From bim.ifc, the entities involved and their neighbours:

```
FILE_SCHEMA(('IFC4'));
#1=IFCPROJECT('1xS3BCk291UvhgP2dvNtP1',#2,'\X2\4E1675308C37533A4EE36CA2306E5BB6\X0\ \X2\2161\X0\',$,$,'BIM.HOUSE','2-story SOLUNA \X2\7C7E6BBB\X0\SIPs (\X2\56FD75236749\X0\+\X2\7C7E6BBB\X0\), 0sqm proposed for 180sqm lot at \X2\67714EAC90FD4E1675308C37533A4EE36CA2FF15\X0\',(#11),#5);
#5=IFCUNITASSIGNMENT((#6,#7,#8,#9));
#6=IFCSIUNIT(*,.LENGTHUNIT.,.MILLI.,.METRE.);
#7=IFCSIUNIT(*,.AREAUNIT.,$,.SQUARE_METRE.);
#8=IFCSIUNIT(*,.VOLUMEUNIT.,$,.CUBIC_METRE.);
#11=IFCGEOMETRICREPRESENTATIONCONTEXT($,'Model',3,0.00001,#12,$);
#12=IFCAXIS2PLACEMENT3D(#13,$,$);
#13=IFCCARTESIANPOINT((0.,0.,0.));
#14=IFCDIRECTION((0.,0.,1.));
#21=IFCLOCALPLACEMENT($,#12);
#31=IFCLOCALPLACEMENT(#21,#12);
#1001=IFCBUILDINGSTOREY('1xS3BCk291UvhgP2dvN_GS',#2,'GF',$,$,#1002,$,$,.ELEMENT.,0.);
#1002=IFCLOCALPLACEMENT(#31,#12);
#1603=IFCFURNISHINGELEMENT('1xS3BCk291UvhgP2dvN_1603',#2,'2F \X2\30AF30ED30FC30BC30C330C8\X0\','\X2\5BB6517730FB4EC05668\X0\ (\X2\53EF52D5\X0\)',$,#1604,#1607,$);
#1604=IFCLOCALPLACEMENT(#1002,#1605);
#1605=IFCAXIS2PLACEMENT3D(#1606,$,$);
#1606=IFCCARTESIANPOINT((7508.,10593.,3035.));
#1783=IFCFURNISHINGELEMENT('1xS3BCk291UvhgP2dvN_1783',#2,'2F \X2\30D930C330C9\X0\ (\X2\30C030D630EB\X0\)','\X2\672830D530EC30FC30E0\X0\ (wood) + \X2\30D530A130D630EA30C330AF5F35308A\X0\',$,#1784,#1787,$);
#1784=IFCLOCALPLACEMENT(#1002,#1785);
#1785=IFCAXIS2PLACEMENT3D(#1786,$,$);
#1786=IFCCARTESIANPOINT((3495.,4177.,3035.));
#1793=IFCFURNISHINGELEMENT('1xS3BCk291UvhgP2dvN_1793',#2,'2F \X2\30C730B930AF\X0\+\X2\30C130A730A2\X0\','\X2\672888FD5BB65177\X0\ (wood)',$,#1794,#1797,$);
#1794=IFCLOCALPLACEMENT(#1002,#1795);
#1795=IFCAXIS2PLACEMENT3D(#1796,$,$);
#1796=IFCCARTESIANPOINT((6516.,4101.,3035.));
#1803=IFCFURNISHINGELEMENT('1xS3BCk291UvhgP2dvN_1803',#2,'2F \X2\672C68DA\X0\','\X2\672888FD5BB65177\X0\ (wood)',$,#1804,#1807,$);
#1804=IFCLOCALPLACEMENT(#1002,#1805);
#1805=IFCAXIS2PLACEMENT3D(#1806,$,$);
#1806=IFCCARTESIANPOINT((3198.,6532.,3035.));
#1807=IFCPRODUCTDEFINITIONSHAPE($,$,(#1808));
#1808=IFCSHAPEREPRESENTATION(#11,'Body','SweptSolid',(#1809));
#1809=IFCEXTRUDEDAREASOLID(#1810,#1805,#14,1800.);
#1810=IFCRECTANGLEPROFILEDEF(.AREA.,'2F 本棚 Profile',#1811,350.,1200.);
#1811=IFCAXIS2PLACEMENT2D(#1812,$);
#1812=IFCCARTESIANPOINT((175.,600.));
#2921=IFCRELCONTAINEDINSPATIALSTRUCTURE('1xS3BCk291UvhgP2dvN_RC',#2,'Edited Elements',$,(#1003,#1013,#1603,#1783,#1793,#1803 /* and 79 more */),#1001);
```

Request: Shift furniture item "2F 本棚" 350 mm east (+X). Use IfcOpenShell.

```python
import ifcopenshell
import ifcopenshell.api.geometry
import ifcopenshell.util.placement

model = ifcopenshell.open("bim.ifc")

item = model.by_id(1803)
matrix = ifcopenshell.util.placement.get_local_placement(item.ObjectPlacement)
matrix[0, 3] += 350.0
ifcopenshell.api.geometry.edit_object_placement(model, product=item, matrix=matrix, is_si=False)

print(ifcopenshell.util.placement.get_local_placement(item.ObjectPlacement).round(3) + 0.0)

model.write("bim_rev.ifc")
```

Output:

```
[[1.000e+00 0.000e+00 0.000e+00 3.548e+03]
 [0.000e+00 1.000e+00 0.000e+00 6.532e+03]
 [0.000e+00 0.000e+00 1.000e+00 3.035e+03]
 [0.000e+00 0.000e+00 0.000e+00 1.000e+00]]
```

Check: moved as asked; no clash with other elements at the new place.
